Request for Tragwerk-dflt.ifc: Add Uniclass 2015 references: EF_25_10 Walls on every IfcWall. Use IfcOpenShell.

First a look at what the model holds.

```python
import ifcopenshell

model = ifcopenshell.open("Tragwerk-dflt.ifc")
print(model.schema)
print("classifications:", [c.Name for c in model.by_type("IfcClassification")])
for ifc_class in ("IfcDoor", "IfcRoof", "IfcStair", "IfcWall", "IfcWindow"):
    print(ifc_class, len(model.by_type(ifc_class)))
```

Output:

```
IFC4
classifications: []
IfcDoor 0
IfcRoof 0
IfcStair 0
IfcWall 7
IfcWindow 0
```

```python
import ifcopenshell
import ifcopenshell.api.classification

model = ifcopenshell.open("Tragwerk-dflt.ifc")

system = ifcopenshell.api.classification.add_classification(model, classification="Uniclass 2015")

codes = {
    "IfcWall": ("EF_25_10", "Walls"),
}
for ifc_class, (code, name) in codes.items():
    products = model.by_type(ifc_class)
    ifcopenshell.api.classification.add_reference(
        model, products=products, classification=system, identification=code, name=name
    )
    print(code, len(products))

model.write("Tragwerk-dflt-out.ifc")
```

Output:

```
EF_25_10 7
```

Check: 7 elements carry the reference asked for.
